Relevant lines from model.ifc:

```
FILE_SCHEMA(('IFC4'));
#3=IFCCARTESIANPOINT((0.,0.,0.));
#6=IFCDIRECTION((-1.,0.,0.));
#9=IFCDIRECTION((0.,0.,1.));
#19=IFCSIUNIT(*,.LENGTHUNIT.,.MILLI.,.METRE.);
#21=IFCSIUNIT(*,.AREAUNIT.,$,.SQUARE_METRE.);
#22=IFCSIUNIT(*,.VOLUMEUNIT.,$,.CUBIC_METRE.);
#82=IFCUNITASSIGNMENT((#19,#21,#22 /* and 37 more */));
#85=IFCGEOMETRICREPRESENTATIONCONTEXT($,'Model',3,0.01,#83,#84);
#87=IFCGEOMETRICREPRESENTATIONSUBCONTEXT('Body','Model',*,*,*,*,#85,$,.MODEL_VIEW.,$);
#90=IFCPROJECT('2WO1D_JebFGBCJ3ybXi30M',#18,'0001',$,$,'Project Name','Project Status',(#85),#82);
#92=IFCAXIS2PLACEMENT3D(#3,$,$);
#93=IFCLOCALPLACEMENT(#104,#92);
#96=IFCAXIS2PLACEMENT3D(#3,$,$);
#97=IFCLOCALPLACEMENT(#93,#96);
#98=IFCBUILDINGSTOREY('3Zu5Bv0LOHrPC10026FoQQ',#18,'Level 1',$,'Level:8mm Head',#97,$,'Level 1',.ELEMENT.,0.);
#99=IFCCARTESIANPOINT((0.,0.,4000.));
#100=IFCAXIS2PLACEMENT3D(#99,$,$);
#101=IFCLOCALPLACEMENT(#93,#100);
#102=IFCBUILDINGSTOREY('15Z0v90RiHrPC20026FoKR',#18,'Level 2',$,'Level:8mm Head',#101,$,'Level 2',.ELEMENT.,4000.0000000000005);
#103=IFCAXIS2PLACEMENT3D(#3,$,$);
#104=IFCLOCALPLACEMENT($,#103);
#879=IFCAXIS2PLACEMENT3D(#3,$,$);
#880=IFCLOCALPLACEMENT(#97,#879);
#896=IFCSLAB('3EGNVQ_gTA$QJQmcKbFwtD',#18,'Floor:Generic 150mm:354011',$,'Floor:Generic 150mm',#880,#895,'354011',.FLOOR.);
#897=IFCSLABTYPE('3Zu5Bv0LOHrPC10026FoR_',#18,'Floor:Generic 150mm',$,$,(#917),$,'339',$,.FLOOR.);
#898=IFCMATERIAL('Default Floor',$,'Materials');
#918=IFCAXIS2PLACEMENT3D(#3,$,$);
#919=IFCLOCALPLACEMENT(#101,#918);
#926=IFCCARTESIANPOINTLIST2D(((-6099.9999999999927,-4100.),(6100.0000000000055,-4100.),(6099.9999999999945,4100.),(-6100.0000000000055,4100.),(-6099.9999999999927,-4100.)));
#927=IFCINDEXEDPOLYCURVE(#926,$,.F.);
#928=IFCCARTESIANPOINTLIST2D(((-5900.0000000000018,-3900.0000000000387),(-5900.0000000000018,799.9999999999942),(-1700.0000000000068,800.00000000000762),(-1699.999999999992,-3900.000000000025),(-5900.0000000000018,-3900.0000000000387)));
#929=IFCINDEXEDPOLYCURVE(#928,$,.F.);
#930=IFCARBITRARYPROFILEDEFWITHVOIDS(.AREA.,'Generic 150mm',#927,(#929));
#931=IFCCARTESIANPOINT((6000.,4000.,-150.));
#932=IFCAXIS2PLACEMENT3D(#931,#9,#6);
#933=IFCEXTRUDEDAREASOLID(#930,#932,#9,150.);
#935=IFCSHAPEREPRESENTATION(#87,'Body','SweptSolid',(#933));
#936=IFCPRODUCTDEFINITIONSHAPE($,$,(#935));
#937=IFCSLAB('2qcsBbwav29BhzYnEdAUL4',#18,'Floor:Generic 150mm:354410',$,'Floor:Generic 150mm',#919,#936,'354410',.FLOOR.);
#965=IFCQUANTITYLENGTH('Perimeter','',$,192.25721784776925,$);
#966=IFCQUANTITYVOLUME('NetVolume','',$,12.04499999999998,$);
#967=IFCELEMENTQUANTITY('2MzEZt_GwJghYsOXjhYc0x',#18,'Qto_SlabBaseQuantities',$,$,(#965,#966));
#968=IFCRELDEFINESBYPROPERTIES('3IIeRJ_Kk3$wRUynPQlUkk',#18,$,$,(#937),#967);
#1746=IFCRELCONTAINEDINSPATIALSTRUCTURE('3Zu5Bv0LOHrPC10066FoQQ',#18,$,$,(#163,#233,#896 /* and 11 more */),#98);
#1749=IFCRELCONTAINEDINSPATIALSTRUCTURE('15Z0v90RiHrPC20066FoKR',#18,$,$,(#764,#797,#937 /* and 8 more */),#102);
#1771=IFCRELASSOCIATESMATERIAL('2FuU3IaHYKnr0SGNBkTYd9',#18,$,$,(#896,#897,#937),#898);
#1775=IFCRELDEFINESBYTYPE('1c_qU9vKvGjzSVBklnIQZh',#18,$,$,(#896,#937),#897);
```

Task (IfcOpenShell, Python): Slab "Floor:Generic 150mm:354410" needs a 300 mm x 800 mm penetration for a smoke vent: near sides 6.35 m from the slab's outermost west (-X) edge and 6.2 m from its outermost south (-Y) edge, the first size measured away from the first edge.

```python
import numpy as np
import ifcopenshell
import ifcopenshell.api.feature
import ifcopenshell.api.geometry
import ifcopenshell.api.pset
import ifcopenshell.api.root
import ifcopenshell.geom
import ifcopenshell.util.element
import ifcopenshell.util.placement
import ifcopenshell.util.representation
import ifcopenshell.util.shape
import ifcopenshell.util.unit

model = ifcopenshell.open("model.ifc")
unit_scale = ifcopenshell.util.unit.calculate_unit_scale(model)
volume_scale = ifcopenshell.util.unit.calculate_unit_scale(model, "VOLUMEUNIT")
settings = ifcopenshell.geom.settings()


def volume(element):
    """Net volume in cubic metres, openings subtracted."""
    shape = ifcopenshell.geom.create_shape(settings, element)
    return ifcopenshell.util.shape.get_volume(shape.geometry)


slab = model.by_guid("2qcsBbwav29BhzYnEdAUL4")
before = volume(slab)

# Extent in the slab's own axes, in metres. The edges named are its -X and -Y sides.
slab_shape = ifcopenshell.geom.create_shape(settings, slab)
vertices = ifcopenshell.util.shape.get_vertices(slab_shape.geometry)
x_min, y_min, bottom = vertices.min(axis=0)
top = vertices[:, 2].max()

opening = ifcopenshell.api.root.create_entity(model, ifc_class="IfcOpeningElement", name="Smoke vent opening", predefined_type="OPENING")
context = ifcopenshell.util.representation.get_context(model, "Model", "Body", "MODEL_VIEW")
width, depth = 0.3, 0.8
outline = [(0.0, 0.0), (width, 0.0), (width, depth), (0.0, depth), (0.0, 0.0)]
# Overshoot both faces by 50 mm so the cut is clean.
shape = ifcopenshell.api.geometry.add_slab_representation(
    model, context=context, depth=top - bottom + 0.1, polyline=outline
)
ifcopenshell.api.geometry.assign_representation(model, product=opening, representation=shape)

matrix = ifcopenshell.util.placement.get_local_placement(slab.ObjectPlacement)
matrix[:, 3] = matrix @ np.append(np.array([x_min + 6.35, y_min + 6.2, bottom - 0.05]) / unit_scale, 1.0)
ifcopenshell.api.geometry.edit_object_placement(model, product=opening, matrix=matrix, is_si=False)
ifcopenshell.api.feature.add_feature(model, feature=opening, element=slab)

after = volume(slab)

# Update the slab's stored quantities.
qto = model.by_id(ifcopenshell.util.element.get_pset(slab, "Qto_SlabBaseQuantities", should_inherit=False)["id"])
ifcopenshell.api.pset.edit_qto(model, qto=qto, properties={"NetVolume": after / volume_scale})

print(f"slab volume {before:.3f} -> {after:.3f} m3")

model.write("model-out.ifc")
```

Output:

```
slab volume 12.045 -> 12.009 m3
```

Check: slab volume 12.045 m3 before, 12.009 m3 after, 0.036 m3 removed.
